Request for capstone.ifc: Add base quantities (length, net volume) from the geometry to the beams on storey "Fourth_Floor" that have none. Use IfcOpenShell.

First a look at what the model holds.

```python
import ifcopenshell
import ifcopenshell.util.element
import ifcopenshell.util.unit

model = ifcopenshell.open("capstone.ifc")
print(model.schema)
for unit_type in ("LENGTHUNIT", "AREAUNIT", "VOLUMEUNIT"):
    print(unit_type, ifcopenshell.util.unit.calculate_unit_scale(model, unit_type))
storey = next(s for s in model.by_type("IfcBuildingStorey") if s.Name == "Fourth_Floor")
beams = [e for e in ifcopenshell.util.element.get_decomposition(storey) if e.is_a("IfcBeam")]
for e in sorted(beams, key=lambda e: e.id()):
    print(e.id(), e.is_a(), e.Name, list(ifcopenshell.util.element.get_psets(e, qtos_only=True)), sep=" | ")
```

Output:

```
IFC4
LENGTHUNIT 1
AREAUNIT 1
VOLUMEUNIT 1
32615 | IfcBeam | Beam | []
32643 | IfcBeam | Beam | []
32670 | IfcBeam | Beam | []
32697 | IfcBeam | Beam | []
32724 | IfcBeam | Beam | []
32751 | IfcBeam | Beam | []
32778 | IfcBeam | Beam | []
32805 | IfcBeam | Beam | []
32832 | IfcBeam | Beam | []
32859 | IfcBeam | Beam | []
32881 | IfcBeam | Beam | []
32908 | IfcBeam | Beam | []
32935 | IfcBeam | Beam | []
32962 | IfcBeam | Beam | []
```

```python
import ifcopenshell
import ifcopenshell.api.pset
import ifcopenshell.geom
import ifcopenshell.util.element
import ifcopenshell.util.shape
import ifcopenshell.util.unit

model = ifcopenshell.open("capstone.ifc")
unit_scale = ifcopenshell.util.unit.calculate_unit_scale(model)
volume_scale = ifcopenshell.util.unit.calculate_unit_scale(model, "VOLUMEUNIT")
settings = ifcopenshell.geom.settings()

storey = next(s for s in model.by_type("IfcBuildingStorey") if s.Name == "Fourth_Floor")
beams = [e for e in ifcopenshell.util.element.get_decomposition(storey) if e.is_a("IfcBeam")]

for e in sorted(beams, key=lambda e: e.id()):
    if ifcopenshell.util.element.get_psets(e, qtos_only=True, should_inherit=False):
        continue
    # Geometry comes back in metres, in the element's own axes.
    shape = ifcopenshell.geom.create_shape(settings, e)
    values = {
        "Length": ifcopenshell.util.shape.get_max_xyz(shape.geometry) / unit_scale,
        "NetVolume": ifcopenshell.util.shape.get_volume(shape.geometry) / volume_scale,
    }
    qto = ifcopenshell.api.pset.add_qto(model, product=e, name="Qto_BeamBaseQuantities")
    ifcopenshell.api.pset.edit_qto(model, qto=qto, properties=values)
    print(e.id(), {k: round(v, 3) for k, v in values.items()})

model.write("capstone_edited.ifc")
```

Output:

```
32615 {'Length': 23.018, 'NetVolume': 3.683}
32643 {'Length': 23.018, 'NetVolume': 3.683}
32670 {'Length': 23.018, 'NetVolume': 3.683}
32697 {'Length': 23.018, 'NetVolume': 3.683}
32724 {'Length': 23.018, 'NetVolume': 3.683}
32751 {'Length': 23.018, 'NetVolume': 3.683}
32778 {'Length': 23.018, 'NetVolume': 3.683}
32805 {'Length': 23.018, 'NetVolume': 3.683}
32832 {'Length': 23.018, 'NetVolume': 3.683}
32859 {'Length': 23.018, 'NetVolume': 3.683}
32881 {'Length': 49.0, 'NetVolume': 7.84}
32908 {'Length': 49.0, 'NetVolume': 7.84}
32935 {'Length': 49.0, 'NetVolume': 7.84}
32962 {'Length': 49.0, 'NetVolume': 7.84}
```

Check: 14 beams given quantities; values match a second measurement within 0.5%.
